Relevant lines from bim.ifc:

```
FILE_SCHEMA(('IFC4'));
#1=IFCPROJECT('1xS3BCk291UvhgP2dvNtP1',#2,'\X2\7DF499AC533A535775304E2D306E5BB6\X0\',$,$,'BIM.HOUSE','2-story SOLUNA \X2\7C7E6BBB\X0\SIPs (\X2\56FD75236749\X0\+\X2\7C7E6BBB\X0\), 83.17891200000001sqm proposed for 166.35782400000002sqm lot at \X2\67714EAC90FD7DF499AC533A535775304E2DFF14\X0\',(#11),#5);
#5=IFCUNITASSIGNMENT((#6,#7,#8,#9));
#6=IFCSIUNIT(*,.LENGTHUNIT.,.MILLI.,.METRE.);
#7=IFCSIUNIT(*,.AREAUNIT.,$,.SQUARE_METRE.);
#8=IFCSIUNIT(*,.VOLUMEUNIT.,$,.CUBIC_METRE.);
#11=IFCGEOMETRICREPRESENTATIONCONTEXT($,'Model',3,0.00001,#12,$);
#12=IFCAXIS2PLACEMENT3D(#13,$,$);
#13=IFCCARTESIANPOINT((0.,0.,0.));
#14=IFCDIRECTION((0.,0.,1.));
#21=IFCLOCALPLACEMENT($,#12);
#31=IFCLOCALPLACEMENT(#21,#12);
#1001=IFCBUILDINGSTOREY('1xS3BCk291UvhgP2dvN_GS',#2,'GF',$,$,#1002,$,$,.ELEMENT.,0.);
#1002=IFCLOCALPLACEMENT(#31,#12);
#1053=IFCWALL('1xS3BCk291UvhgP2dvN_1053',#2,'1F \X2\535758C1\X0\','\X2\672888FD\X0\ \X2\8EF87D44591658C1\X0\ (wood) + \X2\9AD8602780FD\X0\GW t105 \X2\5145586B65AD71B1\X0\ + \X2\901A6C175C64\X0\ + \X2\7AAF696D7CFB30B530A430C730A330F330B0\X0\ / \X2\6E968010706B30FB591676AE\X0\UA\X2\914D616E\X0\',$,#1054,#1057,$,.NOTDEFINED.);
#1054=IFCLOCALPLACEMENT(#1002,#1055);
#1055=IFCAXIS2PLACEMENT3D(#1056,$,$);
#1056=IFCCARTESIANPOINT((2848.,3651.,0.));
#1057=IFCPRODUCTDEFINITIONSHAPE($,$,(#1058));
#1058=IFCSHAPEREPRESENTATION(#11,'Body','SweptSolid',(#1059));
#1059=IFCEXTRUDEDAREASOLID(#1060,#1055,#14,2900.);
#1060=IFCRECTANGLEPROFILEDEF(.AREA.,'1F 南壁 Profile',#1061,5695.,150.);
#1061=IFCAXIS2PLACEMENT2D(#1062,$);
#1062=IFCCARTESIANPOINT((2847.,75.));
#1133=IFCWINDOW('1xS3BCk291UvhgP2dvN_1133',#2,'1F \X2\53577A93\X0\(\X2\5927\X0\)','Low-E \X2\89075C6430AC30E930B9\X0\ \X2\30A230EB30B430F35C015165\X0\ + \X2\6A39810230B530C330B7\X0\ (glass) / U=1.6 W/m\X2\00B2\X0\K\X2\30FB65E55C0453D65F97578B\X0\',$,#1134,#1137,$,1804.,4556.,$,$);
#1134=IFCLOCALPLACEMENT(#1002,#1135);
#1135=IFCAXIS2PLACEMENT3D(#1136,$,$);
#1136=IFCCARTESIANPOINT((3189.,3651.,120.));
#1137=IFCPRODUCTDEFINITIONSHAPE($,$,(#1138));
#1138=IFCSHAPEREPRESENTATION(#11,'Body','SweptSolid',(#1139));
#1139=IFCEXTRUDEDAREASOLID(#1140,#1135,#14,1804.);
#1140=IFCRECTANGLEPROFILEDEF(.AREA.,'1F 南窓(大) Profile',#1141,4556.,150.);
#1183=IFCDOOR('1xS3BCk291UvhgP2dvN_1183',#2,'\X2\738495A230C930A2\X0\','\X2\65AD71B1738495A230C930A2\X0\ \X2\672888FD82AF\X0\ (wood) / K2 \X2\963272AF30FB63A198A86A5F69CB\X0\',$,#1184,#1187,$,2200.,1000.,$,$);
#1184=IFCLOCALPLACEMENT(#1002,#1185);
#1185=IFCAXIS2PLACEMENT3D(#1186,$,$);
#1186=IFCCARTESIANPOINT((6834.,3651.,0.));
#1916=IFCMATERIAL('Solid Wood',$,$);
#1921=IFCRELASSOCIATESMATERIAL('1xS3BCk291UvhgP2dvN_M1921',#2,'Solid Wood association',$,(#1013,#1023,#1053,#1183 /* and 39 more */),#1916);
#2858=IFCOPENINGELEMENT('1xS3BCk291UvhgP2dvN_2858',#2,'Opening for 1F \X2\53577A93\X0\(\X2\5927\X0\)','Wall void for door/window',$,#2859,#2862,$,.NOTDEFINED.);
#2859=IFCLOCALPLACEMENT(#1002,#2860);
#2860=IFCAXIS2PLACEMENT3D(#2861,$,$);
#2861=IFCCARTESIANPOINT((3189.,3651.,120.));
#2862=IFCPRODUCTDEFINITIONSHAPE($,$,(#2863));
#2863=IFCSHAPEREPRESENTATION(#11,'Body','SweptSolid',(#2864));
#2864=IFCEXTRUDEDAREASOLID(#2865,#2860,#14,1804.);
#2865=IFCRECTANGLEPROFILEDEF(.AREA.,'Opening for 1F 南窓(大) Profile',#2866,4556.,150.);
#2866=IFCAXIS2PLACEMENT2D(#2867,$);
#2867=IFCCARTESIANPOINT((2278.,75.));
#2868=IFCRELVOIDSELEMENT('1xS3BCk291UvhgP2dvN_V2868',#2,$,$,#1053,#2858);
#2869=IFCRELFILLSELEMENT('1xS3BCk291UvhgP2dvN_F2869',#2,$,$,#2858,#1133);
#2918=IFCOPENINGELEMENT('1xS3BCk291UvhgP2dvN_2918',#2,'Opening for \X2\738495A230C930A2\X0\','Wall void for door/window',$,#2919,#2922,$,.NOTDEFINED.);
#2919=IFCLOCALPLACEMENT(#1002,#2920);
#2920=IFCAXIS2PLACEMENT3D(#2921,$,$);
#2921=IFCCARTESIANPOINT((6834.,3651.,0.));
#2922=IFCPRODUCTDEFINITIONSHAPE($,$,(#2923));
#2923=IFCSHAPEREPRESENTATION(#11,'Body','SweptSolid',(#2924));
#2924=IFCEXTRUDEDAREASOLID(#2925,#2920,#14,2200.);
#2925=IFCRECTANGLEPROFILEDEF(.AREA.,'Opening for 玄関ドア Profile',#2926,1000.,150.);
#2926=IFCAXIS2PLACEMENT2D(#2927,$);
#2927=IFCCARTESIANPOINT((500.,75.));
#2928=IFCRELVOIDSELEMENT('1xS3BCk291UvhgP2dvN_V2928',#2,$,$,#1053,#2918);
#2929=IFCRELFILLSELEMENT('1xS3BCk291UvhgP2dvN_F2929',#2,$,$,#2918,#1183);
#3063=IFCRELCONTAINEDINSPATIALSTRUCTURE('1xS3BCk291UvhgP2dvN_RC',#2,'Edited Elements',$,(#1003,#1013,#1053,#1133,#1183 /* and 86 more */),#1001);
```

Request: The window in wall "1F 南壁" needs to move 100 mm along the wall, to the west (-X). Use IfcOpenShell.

```python
import ifcopenshell
import ifcopenshell.api.geometry
import ifcopenshell.util.placement
import ifcopenshell.util.unit

model = ifcopenshell.open("bim.ifc")
unit_scale = ifcopenshell.util.unit.calculate_unit_scale(model)

window = model.by_guid("1xS3BCk291UvhgP2dvN_1133")
opening = window.FillsVoids[0].RelatingOpeningElement
wall = opening.VoidsElements[0].RelatingBuildingElement

wall_matrix = ifcopenshell.util.placement.get_local_placement(wall.ObjectPlacement)
shift = wall_matrix[:3, 0] * -0.1 / unit_scale
before = ifcopenshell.util.placement.get_local_placement(window.ObjectPlacement)[:3, 3].copy()

# The window is not placed relative to its opening, so move both.
for product in (opening, window):
    matrix = ifcopenshell.util.placement.get_local_placement(product.ObjectPlacement)
    matrix[:3, 3] += shift
    ifcopenshell.api.geometry.edit_object_placement(model, product=product, matrix=matrix, is_si=False)

after = ifcopenshell.util.placement.get_local_placement(window.ObjectPlacement)[:3, 3]
print("window moved by", (after - before).round(3) + 0.0)

model.write("bim_updated.ifc")
```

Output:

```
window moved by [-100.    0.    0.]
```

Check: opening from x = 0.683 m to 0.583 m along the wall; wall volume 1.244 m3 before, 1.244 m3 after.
